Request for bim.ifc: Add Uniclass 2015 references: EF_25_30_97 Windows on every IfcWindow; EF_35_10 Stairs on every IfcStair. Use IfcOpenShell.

First a look at what the model holds.

```python
import ifcopenshell

model = ifcopenshell.open("bim.ifc")
print(model.schema)
print("classifications:", [c.Name for c in model.by_type("IfcClassification")])
for ifc_class in ("IfcDoor", "IfcRoof", "IfcStair", "IfcWall", "IfcWindow"):
    print(ifc_class, len(model.by_type(ifc_class)))
```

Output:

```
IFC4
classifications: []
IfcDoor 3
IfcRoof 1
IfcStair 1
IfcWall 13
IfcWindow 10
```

```python
import ifcopenshell
import ifcopenshell.api.classification

model = ifcopenshell.open("bim.ifc")

system = ifcopenshell.api.classification.add_classification(model, classification="Uniclass 2015")

codes = {
    "IfcWindow": ("EF_25_30_97", "Windows"),
    "IfcStair": ("EF_35_10", "Stairs"),
}
for ifc_class, (code, name) in codes.items():
    products = model.by_type(ifc_class)
    ifcopenshell.api.classification.add_reference(
        model, products=products, classification=system, identification=code, name=name
    )
    print(code, len(products))

model.write("bim-out.ifc")
```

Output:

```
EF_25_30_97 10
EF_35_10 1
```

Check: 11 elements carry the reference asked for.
